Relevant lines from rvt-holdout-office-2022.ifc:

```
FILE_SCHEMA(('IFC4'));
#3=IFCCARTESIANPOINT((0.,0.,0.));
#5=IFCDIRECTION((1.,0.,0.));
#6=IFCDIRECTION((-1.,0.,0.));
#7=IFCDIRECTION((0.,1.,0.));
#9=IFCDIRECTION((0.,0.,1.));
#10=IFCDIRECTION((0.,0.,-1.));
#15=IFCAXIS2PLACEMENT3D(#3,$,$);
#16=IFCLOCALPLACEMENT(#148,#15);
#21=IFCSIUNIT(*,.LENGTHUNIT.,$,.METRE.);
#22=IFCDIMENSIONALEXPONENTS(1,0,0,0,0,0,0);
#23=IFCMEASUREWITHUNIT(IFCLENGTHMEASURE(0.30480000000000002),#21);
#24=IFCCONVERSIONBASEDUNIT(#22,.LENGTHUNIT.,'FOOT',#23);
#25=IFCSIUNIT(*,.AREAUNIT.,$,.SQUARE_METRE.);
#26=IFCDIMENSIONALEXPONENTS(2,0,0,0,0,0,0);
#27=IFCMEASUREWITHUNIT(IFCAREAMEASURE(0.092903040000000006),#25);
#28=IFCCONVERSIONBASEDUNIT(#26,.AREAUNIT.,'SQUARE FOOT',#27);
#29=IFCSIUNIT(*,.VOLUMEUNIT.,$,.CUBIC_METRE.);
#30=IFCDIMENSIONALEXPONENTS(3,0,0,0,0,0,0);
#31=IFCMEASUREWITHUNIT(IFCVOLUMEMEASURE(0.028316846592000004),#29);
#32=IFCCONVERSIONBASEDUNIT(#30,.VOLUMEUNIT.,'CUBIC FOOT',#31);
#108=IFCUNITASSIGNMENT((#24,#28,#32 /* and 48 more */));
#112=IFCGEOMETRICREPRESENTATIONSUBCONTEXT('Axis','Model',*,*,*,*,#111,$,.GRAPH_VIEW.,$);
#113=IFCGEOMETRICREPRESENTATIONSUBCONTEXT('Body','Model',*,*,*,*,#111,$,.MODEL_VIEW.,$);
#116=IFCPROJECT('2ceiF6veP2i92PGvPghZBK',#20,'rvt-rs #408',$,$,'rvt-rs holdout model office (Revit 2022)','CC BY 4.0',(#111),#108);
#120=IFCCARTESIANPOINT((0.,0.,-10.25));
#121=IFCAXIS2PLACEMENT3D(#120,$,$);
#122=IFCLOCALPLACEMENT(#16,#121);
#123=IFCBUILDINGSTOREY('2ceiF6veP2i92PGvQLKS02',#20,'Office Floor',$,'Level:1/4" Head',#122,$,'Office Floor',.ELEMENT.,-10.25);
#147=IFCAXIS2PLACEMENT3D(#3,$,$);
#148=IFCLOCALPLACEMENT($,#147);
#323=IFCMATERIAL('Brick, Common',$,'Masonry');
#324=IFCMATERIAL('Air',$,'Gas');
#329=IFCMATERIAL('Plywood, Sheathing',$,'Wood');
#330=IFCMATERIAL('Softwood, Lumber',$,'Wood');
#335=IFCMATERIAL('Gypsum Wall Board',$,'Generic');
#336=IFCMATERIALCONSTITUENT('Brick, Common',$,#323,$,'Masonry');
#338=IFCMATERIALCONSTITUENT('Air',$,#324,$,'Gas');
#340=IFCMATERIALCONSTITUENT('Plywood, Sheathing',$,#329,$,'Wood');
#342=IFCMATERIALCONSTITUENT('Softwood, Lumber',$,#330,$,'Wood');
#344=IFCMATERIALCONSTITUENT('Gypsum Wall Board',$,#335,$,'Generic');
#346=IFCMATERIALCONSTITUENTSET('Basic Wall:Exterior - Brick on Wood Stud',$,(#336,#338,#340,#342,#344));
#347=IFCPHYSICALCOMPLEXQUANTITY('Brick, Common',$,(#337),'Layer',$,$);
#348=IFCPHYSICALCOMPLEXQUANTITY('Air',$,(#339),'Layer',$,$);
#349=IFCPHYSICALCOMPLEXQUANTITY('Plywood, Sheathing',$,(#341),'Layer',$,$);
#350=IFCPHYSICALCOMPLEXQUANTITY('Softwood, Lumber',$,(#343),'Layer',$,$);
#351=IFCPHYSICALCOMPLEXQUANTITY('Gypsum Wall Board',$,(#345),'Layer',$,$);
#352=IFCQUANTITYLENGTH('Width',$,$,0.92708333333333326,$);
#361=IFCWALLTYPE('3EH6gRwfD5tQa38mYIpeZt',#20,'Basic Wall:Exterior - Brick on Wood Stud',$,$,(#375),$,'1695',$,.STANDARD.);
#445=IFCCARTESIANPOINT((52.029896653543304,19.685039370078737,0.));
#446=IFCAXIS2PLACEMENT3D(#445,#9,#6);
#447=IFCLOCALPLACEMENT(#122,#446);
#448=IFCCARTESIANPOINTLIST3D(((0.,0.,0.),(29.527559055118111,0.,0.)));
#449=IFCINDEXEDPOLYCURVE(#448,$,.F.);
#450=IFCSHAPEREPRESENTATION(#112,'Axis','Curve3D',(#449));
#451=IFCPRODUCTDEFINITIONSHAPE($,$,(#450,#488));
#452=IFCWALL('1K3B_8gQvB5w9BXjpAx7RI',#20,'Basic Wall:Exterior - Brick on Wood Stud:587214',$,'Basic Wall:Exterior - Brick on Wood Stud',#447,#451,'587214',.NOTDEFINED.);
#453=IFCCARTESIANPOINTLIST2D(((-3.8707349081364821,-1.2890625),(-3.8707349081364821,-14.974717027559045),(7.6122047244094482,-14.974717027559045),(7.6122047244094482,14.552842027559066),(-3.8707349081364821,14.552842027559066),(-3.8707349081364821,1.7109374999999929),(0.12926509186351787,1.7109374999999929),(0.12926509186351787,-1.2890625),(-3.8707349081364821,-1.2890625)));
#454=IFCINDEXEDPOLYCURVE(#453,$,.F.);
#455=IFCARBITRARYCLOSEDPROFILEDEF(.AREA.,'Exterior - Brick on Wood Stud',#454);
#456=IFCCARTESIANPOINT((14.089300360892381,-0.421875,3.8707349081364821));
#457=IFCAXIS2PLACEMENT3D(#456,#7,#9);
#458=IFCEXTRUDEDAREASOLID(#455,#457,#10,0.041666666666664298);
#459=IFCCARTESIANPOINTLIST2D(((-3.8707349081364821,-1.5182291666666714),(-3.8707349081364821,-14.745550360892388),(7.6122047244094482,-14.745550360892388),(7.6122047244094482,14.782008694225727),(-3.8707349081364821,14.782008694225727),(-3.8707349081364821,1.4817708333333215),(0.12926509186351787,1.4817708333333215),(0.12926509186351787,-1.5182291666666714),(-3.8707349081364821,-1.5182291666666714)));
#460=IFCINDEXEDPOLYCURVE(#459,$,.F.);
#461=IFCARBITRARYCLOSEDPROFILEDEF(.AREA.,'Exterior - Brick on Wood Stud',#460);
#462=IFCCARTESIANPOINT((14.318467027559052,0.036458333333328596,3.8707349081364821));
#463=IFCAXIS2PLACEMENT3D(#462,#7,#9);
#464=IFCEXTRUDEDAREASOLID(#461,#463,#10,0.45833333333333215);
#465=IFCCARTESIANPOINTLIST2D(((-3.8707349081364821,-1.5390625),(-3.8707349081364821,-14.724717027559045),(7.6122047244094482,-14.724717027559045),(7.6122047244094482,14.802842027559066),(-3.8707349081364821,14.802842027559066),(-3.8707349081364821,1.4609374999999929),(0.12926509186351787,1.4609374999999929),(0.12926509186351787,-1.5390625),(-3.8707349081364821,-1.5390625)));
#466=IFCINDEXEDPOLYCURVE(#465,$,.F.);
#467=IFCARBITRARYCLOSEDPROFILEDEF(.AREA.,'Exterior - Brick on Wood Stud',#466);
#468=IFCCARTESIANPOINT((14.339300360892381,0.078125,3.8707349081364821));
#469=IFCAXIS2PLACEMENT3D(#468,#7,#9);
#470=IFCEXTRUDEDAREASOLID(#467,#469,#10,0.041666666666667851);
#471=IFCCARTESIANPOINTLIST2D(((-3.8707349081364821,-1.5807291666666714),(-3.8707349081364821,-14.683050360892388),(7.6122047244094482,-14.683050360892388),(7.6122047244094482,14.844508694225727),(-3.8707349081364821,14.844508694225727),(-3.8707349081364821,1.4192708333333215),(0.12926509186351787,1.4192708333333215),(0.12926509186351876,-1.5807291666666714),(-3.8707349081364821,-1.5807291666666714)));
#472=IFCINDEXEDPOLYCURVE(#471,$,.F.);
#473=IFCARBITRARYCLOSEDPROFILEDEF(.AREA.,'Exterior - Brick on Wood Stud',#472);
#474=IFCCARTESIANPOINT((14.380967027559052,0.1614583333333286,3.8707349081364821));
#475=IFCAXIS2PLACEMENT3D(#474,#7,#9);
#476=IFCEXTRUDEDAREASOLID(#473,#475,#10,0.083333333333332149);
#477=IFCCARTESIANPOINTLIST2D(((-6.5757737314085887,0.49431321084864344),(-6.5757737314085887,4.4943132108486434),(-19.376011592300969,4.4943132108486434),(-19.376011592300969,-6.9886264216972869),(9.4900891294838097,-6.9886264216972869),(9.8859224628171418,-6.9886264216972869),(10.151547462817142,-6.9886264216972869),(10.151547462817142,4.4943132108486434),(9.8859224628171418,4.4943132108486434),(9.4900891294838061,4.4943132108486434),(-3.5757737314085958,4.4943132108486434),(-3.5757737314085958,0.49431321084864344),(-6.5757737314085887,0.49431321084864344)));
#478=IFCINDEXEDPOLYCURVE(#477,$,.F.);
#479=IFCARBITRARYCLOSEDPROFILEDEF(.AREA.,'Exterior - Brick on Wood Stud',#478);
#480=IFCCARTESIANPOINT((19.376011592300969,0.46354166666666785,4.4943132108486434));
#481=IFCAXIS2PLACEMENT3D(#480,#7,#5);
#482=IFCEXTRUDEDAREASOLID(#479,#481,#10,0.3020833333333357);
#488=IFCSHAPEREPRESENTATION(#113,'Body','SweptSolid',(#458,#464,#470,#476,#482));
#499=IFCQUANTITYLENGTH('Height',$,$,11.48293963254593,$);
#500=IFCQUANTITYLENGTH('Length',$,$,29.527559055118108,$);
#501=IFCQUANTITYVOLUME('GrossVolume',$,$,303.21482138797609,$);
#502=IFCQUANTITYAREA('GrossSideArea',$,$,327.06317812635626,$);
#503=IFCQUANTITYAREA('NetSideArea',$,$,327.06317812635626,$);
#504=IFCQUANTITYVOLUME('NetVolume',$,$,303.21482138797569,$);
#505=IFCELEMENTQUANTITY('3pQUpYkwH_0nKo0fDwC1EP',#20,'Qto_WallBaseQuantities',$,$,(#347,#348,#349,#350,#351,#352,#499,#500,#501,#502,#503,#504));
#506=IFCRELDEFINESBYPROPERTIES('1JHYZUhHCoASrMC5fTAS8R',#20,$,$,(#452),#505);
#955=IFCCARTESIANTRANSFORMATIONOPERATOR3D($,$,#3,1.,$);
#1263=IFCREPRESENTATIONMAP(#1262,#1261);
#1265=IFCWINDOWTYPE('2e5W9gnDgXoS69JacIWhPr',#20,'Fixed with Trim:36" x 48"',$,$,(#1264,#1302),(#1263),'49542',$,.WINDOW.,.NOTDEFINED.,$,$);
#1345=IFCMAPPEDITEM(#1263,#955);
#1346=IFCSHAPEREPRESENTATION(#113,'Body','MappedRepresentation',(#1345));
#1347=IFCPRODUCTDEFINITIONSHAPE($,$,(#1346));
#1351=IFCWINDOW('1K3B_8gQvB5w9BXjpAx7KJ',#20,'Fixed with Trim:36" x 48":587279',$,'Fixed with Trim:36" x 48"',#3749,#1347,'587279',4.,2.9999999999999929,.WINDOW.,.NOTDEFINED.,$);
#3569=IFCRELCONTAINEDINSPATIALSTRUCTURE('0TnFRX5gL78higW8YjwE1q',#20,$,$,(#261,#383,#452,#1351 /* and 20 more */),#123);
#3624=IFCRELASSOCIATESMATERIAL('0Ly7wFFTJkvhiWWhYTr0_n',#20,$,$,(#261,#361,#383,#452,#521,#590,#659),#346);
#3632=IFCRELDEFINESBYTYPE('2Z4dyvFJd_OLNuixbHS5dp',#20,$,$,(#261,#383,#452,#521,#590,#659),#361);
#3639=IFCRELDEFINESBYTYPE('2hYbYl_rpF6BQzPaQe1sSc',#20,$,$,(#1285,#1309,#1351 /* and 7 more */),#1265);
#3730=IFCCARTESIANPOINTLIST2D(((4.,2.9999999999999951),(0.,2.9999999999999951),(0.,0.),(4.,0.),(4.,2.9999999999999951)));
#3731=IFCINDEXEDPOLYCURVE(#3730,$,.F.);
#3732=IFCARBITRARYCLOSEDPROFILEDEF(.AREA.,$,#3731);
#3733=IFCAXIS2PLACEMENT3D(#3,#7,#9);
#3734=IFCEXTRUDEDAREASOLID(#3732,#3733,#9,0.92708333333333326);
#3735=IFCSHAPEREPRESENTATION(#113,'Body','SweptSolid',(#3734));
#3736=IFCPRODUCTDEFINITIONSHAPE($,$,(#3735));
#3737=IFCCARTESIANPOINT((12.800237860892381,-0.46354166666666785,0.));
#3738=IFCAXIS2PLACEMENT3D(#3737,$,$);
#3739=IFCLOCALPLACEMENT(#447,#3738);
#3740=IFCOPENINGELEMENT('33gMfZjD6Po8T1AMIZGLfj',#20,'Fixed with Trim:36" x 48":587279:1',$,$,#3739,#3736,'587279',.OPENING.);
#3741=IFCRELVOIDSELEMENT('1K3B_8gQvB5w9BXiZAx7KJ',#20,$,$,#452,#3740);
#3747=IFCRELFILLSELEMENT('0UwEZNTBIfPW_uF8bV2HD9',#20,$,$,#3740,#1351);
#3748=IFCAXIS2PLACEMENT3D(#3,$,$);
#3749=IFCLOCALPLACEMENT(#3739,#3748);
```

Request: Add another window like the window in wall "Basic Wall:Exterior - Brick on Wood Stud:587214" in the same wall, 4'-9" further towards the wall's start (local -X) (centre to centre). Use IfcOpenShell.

```python
import ifcopenshell
import ifcopenshell.api.feature
import ifcopenshell.api.geometry
import ifcopenshell.api.pset
import ifcopenshell.api.root
import ifcopenshell.geom
import ifcopenshell.util.element
import ifcopenshell.util.placement
import ifcopenshell.util.shape
import ifcopenshell.util.unit

model = ifcopenshell.open("rvt-holdout-office-2022.ifc")
unit_scale = ifcopenshell.util.unit.calculate_unit_scale(model)
area_scale = ifcopenshell.util.unit.calculate_unit_scale(model, "AREAUNIT")
volume_scale = ifcopenshell.util.unit.calculate_unit_scale(model, "VOLUMEUNIT")
settings = ifcopenshell.geom.settings()


def volume(element):
    """Net volume in cubic metres, openings subtracted."""
    shape = ifcopenshell.geom.create_shape(settings, element)
    return ifcopenshell.util.shape.get_volume(shape.geometry)


def reuse_history(source, copy):
    """copy_class also copies each property set's owner history, people and application; keep the originals."""
    for rel in copy.IsDefinedBy:
        if rel.is_a("IfcRelDefinesByProperties") and (history := rel.RelatingPropertyDefinition.OwnerHistory):
            rel.RelatingPropertyDefinition.OwnerHistory = source.OwnerHistory
            ifcopenshell.util.element.remove_deep2(model, history)


window = model.by_guid("1K3B_8gQvB5w9BXjpAx7KJ")
opening = window.FillsVoids[0].RelatingOpeningElement
wall = opening.VoidsElements[0].RelatingBuildingElement
before = volume(wall)
shift = ifcopenshell.util.placement.get_local_placement(wall.ObjectPlacement)[:3, 0] * -57 * 0.0254 / unit_scale

# copy_class copies the void relationship, type, container and properties, but no geometry.
new_opening = ifcopenshell.api.root.copy_class(model, product=opening)
new_opening.Representation = ifcopenshell.util.element.copy_deep(
    model, opening.Representation, exclude=["IfcGeometricRepresentationContext", "IfcRepresentationMap"]
)
new_opening.Name = 'Fixed with Trim:36" x 48"'
new_opening.Tag = None
reuse_history(opening, new_opening)
new_window = ifcopenshell.api.root.copy_class(model, product=window)
new_window.Representation = ifcopenshell.util.element.copy_deep(
    model, window.Representation, exclude=["IfcGeometricRepresentationContext", "IfcRepresentationMap"]
)
new_window.Name = 'Fixed with Trim:36" x 48"'
new_window.Tag = None
reuse_history(window, new_window)
ifcopenshell.api.feature.add_filling(model, opening=new_opening, element=new_window)

for old, new in ((opening, new_opening), (window, new_window)):
    matrix = ifcopenshell.util.placement.get_local_placement(old.ObjectPlacement)
    matrix[:3, 3] += shift
    ifcopenshell.api.geometry.edit_object_placement(model, product=new, matrix=matrix, is_si=False)

after = volume(wall)
thickness = 0.2826  # wall thickness in metres

# Update the wall's stored quantities.
qto = model.by_id(ifcopenshell.util.element.get_pset(wall, "Qto_WallBaseQuantities", should_inherit=False)["id"])
ifcopenshell.api.pset.edit_qto(model, qto=qto, properties={
    "NetSideArea": after / thickness / area_scale,
    "NetVolume": after / volume_scale,
})

print(f"wall volume {before:.3f} -> {after:.3f} m3")

model.write("rvt-holdout-office-2022_updated.ifc")
```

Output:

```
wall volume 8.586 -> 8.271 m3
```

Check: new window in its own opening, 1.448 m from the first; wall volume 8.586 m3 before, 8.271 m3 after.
